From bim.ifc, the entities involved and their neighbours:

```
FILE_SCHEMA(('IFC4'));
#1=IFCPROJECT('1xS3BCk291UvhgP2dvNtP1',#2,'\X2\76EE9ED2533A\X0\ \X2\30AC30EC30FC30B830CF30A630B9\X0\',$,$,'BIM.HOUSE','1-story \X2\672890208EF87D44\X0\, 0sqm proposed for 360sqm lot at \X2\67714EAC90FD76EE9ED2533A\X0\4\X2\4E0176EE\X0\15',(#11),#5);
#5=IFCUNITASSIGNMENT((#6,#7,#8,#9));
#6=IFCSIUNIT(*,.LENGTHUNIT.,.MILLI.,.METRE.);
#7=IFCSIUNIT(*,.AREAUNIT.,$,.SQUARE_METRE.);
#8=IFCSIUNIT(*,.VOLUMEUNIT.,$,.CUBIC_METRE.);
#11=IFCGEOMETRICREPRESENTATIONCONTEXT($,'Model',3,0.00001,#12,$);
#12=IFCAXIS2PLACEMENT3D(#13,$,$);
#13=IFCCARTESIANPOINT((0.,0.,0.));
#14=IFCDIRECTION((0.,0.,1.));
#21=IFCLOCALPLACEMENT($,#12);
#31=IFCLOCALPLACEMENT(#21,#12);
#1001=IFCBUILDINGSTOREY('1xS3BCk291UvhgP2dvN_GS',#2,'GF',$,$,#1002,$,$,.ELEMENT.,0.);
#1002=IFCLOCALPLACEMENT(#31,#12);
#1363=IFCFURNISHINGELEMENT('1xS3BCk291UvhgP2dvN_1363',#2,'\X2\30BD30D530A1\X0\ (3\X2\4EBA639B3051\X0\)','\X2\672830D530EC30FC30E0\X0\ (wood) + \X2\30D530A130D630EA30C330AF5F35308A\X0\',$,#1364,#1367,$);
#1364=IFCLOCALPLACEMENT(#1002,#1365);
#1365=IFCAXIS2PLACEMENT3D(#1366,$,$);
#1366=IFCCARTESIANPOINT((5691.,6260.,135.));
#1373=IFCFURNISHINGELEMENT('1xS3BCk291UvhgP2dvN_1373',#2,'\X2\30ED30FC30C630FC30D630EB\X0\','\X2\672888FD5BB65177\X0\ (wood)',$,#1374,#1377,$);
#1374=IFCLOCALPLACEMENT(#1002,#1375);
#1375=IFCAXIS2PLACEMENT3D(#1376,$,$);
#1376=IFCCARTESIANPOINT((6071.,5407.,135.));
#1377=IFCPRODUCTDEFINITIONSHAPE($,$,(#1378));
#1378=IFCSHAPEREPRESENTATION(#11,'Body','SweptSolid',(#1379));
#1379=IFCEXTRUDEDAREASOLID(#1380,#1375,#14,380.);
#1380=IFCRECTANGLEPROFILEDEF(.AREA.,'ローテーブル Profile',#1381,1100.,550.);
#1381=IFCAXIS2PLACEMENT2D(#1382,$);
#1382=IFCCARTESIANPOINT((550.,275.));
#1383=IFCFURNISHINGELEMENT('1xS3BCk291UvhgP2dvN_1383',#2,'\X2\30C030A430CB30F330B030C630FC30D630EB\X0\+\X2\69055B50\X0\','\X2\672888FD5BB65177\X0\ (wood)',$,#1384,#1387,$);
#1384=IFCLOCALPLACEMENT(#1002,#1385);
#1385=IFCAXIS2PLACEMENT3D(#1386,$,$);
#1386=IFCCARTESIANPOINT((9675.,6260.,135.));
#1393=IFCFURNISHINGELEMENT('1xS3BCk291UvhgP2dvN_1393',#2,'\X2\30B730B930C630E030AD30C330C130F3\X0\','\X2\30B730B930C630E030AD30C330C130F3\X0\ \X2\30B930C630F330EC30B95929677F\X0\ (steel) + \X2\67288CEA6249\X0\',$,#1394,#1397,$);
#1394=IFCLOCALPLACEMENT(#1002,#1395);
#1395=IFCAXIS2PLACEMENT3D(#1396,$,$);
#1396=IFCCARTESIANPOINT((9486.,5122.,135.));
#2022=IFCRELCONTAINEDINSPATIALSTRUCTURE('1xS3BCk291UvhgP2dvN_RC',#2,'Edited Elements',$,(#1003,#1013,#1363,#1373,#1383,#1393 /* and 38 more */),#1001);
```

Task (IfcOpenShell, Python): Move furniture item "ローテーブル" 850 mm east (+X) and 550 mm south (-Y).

```python
import ifcopenshell
import ifcopenshell.api.geometry
import ifcopenshell.util.placement
import ifcopenshell.util.unit

model = ifcopenshell.open("bim.ifc")
unit_scale = ifcopenshell.util.unit.calculate_unit_scale(model)

item = model.by_guid("1xS3BCk291UvhgP2dvN_1373")
matrix = ifcopenshell.util.placement.get_local_placement(item.ObjectPlacement)
matrix[0, 3] += 0.85 / unit_scale
matrix[1, 3] -= 0.55 / unit_scale
ifcopenshell.api.geometry.edit_object_placement(model, product=item, matrix=matrix, is_si=False)

print(ifcopenshell.util.placement.get_local_placement(item.ObjectPlacement).round(3) + 0.0)

model.write("bim-out.ifc")
```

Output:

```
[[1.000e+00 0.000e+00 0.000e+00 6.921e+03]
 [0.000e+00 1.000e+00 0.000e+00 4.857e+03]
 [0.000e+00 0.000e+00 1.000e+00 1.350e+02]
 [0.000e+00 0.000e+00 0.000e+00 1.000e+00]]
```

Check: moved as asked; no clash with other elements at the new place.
